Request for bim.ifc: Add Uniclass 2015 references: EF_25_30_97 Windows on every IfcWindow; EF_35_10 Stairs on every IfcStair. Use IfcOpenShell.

First a look at what the model holds.

```python
import ifcopenshell

model = ifcopenshell.open("bim.ifc")
print(model.schema)
print("classifications:", [c.Name for c in model.by_type("IfcClassification")])
for ifc_class in ("IfcDoor", "IfcRoof", "IfcStair", "IfcWall", "IfcWindow"):
    print(ifc_class, len(model.by_type(ifc_class)))
```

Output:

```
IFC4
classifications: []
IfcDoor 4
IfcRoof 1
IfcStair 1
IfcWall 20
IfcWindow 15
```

```python
import ifcopenshell
import ifcopenshell.api.classification

model = ifcopenshell.open("bim.ifc")

system = ifcopenshell.api.classification.add_classification(model, classification="Uniclass 2015")

codes = {
    "IfcWindow": ("EF_25_30_97", "Windows"),
    "IfcStair": ("EF_35_10", "Stairs"),
}
for ifc_class, (code, name) in codes.items():
    products = model.by_type(ifc_class)
    ifcopenshell.api.classification.add_reference(
        model, products=products, classification=system, identification=code, name=name
    )
    print(code, len(products))

model.write("bim_v2.ifc")
```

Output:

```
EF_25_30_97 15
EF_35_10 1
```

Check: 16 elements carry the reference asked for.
